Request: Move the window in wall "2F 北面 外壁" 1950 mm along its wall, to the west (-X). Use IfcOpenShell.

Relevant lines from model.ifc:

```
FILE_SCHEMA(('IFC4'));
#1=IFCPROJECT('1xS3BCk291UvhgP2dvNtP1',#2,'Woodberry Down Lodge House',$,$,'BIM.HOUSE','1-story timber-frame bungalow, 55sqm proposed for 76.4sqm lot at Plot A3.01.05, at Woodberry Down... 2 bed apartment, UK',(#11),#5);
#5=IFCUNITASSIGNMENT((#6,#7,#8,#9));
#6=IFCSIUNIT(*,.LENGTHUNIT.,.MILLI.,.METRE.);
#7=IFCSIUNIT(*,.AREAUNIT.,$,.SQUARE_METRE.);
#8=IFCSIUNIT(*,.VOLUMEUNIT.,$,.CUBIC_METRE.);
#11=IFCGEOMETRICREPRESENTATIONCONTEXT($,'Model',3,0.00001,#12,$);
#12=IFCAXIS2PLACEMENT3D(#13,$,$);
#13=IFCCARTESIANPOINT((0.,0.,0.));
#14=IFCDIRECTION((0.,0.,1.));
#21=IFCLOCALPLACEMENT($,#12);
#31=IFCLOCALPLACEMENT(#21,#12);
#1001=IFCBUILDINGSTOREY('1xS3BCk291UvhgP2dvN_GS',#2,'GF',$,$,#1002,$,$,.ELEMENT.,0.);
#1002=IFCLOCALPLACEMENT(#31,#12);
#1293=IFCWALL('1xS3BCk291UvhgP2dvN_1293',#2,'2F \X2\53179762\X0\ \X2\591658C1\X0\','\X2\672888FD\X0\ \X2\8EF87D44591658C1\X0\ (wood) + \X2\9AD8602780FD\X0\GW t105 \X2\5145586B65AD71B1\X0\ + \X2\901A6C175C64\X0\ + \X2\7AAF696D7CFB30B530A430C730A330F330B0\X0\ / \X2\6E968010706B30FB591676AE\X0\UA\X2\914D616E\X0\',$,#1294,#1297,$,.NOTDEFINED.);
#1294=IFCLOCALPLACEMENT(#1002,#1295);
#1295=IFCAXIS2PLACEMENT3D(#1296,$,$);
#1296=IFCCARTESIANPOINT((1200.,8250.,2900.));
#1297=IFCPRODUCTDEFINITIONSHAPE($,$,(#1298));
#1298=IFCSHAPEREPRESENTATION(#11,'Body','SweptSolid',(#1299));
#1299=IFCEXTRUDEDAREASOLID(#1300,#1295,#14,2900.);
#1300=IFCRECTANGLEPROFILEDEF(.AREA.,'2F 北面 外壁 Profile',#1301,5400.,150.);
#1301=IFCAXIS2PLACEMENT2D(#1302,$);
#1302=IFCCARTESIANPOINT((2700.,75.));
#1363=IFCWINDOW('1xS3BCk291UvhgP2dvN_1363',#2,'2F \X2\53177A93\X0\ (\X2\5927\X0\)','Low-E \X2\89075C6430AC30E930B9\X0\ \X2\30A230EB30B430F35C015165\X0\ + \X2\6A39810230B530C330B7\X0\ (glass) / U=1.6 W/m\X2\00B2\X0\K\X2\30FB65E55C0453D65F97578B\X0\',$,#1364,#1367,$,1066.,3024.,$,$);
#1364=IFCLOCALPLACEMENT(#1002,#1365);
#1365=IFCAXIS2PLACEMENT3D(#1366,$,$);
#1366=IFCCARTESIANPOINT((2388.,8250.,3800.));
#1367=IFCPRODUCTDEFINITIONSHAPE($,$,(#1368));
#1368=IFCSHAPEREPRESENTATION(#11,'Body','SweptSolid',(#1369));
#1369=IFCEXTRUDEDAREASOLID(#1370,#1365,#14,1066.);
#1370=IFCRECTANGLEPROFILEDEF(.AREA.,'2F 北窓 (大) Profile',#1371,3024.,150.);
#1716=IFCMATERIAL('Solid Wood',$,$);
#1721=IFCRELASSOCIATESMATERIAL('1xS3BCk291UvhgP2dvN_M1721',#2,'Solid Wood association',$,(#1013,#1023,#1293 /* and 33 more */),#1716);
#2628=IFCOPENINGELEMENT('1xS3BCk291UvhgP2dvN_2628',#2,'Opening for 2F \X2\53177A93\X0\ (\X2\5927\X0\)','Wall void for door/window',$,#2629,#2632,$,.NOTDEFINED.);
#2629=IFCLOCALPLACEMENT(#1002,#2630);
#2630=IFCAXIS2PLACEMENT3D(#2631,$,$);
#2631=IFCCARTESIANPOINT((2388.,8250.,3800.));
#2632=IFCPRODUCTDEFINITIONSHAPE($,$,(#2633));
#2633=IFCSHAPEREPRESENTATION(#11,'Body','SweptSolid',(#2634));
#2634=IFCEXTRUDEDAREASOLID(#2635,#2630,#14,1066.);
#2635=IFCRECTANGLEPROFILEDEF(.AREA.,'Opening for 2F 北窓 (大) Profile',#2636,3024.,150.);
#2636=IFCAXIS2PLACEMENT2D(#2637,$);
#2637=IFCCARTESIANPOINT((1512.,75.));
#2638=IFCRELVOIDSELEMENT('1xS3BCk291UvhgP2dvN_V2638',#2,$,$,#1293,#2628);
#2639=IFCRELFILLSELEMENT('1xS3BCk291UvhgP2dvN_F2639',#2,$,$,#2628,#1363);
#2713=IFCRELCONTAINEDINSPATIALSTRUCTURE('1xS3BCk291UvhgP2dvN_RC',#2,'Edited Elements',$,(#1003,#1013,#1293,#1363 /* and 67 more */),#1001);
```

```python
import ifcopenshell
import ifcopenshell.api.geometry
import ifcopenshell.util.placement
import ifcopenshell.util.unit

model = ifcopenshell.open("model.ifc")
unit_scale = ifcopenshell.util.unit.calculate_unit_scale(model)

window = model.by_guid("1xS3BCk291UvhgP2dvN_1363")
opening = window.FillsVoids[0].RelatingOpeningElement
wall = opening.VoidsElements[0].RelatingBuildingElement

wall_matrix = ifcopenshell.util.placement.get_local_placement(wall.ObjectPlacement)
shift = wall_matrix[:3, 0] * -1.95 / unit_scale
before = ifcopenshell.util.placement.get_local_placement(window.ObjectPlacement)[:3, 3].copy()

# The window is not placed relative to its opening, so move both.
for product in (opening, window):
    matrix = ifcopenshell.util.placement.get_local_placement(product.ObjectPlacement)
    matrix[:3, 3] += shift
    ifcopenshell.api.geometry.edit_object_placement(model, product=product, matrix=matrix, is_si=False)

after = ifcopenshell.util.placement.get_local_placement(window.ObjectPlacement)[:3, 3]
print("window moved by", (after - before).round(3) + 0.0)

model.write("model_rev.ifc")
```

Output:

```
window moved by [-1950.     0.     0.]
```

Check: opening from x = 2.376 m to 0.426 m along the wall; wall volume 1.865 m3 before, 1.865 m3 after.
